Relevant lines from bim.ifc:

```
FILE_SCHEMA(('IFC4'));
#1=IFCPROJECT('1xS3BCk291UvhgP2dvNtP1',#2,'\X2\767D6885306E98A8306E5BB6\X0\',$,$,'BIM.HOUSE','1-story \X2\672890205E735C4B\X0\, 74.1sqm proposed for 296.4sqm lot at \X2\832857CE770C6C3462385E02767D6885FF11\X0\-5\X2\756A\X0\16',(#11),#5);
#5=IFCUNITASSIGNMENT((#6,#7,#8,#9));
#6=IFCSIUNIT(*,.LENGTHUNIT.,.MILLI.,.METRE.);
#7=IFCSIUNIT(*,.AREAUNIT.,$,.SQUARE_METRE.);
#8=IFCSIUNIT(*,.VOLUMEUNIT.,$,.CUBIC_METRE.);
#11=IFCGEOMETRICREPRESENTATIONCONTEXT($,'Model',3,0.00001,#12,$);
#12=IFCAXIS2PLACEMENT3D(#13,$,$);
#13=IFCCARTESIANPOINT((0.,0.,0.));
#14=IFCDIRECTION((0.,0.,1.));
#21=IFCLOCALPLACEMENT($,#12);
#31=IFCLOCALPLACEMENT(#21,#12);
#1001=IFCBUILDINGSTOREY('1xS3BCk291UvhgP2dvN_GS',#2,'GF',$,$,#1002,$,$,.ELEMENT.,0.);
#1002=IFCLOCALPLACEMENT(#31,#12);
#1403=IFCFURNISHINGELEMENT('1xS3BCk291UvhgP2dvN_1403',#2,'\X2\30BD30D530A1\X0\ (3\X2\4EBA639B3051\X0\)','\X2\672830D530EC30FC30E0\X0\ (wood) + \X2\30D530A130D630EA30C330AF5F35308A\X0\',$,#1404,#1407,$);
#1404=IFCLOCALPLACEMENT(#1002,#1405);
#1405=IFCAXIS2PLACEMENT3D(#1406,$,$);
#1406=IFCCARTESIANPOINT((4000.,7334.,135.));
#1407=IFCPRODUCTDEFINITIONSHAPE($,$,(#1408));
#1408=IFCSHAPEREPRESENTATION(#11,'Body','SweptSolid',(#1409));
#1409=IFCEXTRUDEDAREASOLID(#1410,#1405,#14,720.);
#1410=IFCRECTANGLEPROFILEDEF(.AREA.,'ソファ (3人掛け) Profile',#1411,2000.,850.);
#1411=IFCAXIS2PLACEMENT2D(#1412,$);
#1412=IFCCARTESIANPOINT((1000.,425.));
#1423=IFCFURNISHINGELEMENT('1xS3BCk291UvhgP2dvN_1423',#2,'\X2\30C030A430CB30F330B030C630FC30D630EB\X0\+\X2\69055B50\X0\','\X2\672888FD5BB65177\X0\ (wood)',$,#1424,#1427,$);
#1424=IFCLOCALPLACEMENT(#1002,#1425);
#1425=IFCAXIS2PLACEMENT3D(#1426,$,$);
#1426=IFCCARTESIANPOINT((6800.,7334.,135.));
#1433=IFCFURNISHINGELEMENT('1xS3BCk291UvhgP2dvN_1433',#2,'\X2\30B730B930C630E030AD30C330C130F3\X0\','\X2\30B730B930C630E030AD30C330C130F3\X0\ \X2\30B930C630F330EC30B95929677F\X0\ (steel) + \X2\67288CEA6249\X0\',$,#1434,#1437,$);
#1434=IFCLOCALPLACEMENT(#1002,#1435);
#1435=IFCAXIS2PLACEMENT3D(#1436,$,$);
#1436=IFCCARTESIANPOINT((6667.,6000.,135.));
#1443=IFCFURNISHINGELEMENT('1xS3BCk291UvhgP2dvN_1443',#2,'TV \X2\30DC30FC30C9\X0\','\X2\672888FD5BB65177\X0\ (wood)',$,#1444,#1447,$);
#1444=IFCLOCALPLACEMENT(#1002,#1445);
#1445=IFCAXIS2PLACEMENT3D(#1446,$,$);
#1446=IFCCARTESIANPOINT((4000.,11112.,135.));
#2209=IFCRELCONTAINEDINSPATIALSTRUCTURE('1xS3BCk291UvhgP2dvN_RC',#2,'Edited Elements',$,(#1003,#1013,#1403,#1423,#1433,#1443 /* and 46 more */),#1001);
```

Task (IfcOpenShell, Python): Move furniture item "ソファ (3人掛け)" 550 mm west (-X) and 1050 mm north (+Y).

```python
import ifcopenshell
import ifcopenshell.api.geometry
import ifcopenshell.util.placement
import ifcopenshell.util.unit

model = ifcopenshell.open("bim.ifc")
unit_scale = ifcopenshell.util.unit.calculate_unit_scale(model)

item = model.by_guid("1xS3BCk291UvhgP2dvN_1403")
matrix = ifcopenshell.util.placement.get_local_placement(item.ObjectPlacement)
matrix[0, 3] -= 0.55 / unit_scale
matrix[1, 3] += 1.05 / unit_scale
ifcopenshell.api.geometry.edit_object_placement(model, product=item, matrix=matrix, is_si=False)

print(ifcopenshell.util.placement.get_local_placement(item.ObjectPlacement).round(3) + 0.0)

model.write("bim_updated.ifc")
```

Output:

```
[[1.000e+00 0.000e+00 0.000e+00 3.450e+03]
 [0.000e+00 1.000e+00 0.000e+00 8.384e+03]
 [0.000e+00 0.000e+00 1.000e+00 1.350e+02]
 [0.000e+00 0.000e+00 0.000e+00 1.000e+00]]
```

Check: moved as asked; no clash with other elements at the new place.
